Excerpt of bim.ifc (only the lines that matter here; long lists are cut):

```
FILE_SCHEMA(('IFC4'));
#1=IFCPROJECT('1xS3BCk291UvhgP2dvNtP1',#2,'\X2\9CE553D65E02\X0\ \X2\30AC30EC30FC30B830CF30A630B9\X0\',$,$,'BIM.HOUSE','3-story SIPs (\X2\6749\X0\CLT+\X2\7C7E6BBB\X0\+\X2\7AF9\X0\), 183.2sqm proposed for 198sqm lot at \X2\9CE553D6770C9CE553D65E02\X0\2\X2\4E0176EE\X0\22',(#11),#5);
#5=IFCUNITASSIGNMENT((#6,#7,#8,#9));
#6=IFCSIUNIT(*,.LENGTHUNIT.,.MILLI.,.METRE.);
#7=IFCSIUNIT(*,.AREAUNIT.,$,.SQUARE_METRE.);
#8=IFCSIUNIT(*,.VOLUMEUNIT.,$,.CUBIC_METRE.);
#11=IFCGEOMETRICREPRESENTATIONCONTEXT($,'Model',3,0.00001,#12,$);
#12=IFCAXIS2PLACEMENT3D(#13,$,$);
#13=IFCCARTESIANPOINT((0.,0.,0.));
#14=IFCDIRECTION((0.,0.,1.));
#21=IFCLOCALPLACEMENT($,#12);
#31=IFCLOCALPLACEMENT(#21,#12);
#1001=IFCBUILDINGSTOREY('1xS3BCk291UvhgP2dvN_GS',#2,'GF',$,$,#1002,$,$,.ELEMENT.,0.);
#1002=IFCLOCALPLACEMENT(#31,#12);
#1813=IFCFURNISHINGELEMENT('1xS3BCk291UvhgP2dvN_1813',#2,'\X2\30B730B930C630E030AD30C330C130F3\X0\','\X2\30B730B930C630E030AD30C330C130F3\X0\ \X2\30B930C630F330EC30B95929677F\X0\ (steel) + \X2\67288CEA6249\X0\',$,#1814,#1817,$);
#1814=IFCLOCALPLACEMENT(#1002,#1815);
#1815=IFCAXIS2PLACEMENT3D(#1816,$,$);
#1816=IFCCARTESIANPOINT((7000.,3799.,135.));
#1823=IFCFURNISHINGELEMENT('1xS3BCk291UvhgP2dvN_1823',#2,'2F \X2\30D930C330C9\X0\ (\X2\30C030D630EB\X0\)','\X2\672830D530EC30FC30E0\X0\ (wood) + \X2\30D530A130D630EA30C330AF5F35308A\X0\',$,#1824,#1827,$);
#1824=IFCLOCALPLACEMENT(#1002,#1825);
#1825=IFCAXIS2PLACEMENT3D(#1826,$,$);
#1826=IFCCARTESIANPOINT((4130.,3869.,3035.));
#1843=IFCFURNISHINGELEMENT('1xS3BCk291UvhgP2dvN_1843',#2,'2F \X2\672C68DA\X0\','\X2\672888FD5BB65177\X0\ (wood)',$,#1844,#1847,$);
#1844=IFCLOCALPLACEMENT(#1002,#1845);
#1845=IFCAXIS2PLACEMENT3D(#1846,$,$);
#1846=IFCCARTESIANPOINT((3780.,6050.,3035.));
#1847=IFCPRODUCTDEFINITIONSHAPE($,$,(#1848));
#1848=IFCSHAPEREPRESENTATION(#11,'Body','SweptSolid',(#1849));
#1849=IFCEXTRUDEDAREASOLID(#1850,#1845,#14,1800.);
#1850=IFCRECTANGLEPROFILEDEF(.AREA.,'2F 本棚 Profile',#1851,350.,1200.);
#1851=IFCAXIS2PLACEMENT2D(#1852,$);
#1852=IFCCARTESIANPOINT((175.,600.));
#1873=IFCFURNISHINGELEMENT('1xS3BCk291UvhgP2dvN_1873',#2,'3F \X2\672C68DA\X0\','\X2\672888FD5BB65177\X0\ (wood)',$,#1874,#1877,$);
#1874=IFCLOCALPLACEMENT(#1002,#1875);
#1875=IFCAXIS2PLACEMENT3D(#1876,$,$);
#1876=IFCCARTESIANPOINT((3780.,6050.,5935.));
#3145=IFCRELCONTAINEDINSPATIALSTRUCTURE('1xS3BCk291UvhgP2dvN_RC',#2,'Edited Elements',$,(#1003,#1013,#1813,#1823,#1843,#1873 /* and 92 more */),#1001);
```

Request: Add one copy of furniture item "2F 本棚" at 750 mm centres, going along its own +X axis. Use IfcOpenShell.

```python
import ifcopenshell
import ifcopenshell.api.geometry
import ifcopenshell.api.root
import ifcopenshell.util.element
import ifcopenshell.util.placement

model = ifcopenshell.open("bim.ifc")


def reuse_history(source, copy):
    """copy_class also copies each property set's owner history, people and application; keep the originals."""
    for rel in copy.IsDefinedBy:
        if rel.is_a("IfcRelDefinesByProperties") and (history := rel.RelatingPropertyDefinition.OwnerHistory):
            rel.RelatingPropertyDefinition.OwnerHistory = source.OwnerHistory
            ifcopenshell.util.element.remove_deep2(model, history)


source = model.by_guid("1xS3BCk291UvhgP2dvN_1843")
base = ifcopenshell.util.placement.get_local_placement(source.ObjectPlacement)
step = base[:3, 0] * 750.0

for i in range(1, 2):
    copy = ifcopenshell.api.root.copy_class(model, product=source)
    copy.Representation = ifcopenshell.util.element.copy_deep(
        model, source.Representation, exclude=["IfcGeometricRepresentationContext", "IfcRepresentationMap"]
    )
    reuse_history(source, copy)
    matrix = base.copy()
    matrix[:3, 3] += i * step
    print("added at", matrix[:3, 3].round(3) + 0.0)
    ifcopenshell.api.geometry.edit_object_placement(model, product=copy, matrix=matrix, is_si=False)

model.write("bim_rev.ifc")
```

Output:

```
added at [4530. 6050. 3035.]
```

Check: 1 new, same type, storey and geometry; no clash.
